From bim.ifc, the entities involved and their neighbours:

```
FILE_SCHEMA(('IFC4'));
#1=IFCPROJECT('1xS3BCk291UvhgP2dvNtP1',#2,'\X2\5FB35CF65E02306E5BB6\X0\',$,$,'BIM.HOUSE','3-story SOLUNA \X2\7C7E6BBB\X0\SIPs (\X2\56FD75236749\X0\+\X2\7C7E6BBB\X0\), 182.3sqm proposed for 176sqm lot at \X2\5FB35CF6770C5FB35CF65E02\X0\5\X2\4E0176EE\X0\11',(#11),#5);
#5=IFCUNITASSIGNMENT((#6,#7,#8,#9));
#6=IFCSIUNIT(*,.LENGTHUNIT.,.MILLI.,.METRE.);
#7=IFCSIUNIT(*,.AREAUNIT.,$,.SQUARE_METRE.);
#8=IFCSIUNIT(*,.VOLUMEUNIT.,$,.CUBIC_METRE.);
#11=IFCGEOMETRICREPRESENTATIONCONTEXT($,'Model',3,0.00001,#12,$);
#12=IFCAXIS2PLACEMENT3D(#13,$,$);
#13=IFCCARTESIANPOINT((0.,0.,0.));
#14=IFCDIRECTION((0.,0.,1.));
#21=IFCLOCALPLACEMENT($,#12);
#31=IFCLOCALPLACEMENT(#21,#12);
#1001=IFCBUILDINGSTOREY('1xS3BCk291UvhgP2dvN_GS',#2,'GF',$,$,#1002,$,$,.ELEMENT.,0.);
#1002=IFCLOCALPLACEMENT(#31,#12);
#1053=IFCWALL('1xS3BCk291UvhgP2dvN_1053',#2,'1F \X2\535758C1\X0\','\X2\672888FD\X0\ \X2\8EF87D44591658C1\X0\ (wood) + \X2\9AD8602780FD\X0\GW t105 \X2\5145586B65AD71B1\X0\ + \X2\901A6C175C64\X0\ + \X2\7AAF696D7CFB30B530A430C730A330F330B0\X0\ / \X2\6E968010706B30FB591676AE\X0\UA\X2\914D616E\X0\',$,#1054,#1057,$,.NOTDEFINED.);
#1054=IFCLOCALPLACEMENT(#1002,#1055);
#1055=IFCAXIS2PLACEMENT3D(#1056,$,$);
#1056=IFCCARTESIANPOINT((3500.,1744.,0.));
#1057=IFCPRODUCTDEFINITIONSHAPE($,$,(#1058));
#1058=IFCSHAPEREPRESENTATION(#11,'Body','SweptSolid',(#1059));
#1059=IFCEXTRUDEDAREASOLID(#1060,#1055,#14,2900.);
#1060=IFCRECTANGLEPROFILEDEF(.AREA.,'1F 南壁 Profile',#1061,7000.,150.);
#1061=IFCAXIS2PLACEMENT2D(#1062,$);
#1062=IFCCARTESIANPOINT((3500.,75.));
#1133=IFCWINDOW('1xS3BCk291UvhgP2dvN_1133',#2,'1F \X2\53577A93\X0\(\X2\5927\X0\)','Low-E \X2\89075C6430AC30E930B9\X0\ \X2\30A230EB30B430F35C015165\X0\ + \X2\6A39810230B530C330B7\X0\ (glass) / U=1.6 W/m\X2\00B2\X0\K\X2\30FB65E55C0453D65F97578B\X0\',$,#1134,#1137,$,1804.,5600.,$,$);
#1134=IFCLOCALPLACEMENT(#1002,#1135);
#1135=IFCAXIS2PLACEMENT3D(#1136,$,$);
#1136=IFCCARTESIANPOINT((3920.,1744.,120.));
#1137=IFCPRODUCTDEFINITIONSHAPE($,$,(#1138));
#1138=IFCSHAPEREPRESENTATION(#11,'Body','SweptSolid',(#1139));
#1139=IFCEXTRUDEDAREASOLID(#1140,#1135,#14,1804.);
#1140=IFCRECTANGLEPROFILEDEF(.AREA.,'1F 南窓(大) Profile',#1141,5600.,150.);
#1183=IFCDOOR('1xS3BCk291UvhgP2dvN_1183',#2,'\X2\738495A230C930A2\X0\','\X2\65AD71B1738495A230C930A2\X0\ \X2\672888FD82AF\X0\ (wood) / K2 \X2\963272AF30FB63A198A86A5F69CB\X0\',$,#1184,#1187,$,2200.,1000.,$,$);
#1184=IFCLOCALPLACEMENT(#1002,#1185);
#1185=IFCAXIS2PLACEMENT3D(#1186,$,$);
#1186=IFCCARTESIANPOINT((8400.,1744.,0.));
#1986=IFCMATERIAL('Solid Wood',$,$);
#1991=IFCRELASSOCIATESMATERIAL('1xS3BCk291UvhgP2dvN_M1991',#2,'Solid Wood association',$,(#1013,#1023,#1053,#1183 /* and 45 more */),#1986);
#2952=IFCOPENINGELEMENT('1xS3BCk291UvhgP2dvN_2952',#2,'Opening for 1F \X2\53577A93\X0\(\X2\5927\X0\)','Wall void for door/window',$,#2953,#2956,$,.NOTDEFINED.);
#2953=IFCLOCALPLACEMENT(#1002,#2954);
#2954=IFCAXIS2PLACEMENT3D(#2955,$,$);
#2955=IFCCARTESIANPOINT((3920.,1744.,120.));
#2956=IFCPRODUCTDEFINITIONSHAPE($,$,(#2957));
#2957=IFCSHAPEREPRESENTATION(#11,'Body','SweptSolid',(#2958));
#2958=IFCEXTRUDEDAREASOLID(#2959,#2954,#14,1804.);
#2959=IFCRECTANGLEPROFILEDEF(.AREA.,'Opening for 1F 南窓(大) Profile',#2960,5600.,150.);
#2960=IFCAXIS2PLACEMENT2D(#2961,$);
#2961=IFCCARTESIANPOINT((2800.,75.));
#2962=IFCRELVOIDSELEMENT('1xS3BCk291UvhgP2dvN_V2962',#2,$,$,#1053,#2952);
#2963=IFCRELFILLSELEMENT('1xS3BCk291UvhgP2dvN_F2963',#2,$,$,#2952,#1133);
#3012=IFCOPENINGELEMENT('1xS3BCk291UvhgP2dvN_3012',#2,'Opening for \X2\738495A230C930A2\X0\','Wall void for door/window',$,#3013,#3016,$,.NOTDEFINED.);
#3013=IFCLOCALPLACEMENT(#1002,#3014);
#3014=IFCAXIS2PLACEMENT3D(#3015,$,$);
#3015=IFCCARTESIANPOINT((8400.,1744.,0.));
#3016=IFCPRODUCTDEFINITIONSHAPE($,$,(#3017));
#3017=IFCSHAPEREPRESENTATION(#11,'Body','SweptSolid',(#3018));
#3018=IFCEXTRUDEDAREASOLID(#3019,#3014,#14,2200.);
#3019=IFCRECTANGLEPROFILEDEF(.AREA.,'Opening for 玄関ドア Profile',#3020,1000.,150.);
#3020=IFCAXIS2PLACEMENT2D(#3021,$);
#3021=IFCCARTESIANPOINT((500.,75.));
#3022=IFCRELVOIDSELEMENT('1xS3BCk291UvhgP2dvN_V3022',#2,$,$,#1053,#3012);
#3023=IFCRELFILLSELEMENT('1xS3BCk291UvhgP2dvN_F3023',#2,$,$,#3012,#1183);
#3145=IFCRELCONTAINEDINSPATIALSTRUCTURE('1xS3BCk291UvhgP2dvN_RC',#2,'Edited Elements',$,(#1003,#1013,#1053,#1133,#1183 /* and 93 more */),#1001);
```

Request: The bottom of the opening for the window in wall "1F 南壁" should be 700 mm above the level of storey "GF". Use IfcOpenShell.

```python
import numpy as np
import ifcopenshell
import ifcopenshell.api.geometry
import ifcopenshell.geom
import ifcopenshell.util.element
import ifcopenshell.util.placement
import ifcopenshell.util.shape
import ifcopenshell.util.unit

model = ifcopenshell.open("bim.ifc")
unit_scale = ifcopenshell.util.unit.calculate_unit_scale(model)

window = model.by_guid("1xS3BCk291UvhgP2dvN_1133")
opening = window.FillsVoids[0].RelatingOpeningElement
storey = ifcopenshell.util.element.get_container(window, ifc_class="IfcBuildingStorey")
level = ifcopenshell.util.placement.get_local_placement(storey.ObjectPlacement)[2, 3]

# The opening's origin need not be at the sill, so measure its lowest point.
shape = ifcopenshell.geom.create_shape(ifcopenshell.geom.settings(), opening)
bottom = ifcopenshell.util.shape.get_shape_bottom_elevation(shape, shape.geometry) / unit_scale
dz = level + 0.7 / unit_scale - bottom

shift = np.array([0.0, 0.0, dz])
# The window is not placed relative to its opening, so move both.
for product in (opening, window):
    matrix = ifcopenshell.util.placement.get_local_placement(product.ObjectPlacement)
    matrix[:3, 3] += shift
    ifcopenshell.api.geometry.edit_object_placement(model, product=product, matrix=matrix, is_si=False)

print(f"moved by {dz * unit_scale:+.3f} m")

model.write("bim-out.ifc")
```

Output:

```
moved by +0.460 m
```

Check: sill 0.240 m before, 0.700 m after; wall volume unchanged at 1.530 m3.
